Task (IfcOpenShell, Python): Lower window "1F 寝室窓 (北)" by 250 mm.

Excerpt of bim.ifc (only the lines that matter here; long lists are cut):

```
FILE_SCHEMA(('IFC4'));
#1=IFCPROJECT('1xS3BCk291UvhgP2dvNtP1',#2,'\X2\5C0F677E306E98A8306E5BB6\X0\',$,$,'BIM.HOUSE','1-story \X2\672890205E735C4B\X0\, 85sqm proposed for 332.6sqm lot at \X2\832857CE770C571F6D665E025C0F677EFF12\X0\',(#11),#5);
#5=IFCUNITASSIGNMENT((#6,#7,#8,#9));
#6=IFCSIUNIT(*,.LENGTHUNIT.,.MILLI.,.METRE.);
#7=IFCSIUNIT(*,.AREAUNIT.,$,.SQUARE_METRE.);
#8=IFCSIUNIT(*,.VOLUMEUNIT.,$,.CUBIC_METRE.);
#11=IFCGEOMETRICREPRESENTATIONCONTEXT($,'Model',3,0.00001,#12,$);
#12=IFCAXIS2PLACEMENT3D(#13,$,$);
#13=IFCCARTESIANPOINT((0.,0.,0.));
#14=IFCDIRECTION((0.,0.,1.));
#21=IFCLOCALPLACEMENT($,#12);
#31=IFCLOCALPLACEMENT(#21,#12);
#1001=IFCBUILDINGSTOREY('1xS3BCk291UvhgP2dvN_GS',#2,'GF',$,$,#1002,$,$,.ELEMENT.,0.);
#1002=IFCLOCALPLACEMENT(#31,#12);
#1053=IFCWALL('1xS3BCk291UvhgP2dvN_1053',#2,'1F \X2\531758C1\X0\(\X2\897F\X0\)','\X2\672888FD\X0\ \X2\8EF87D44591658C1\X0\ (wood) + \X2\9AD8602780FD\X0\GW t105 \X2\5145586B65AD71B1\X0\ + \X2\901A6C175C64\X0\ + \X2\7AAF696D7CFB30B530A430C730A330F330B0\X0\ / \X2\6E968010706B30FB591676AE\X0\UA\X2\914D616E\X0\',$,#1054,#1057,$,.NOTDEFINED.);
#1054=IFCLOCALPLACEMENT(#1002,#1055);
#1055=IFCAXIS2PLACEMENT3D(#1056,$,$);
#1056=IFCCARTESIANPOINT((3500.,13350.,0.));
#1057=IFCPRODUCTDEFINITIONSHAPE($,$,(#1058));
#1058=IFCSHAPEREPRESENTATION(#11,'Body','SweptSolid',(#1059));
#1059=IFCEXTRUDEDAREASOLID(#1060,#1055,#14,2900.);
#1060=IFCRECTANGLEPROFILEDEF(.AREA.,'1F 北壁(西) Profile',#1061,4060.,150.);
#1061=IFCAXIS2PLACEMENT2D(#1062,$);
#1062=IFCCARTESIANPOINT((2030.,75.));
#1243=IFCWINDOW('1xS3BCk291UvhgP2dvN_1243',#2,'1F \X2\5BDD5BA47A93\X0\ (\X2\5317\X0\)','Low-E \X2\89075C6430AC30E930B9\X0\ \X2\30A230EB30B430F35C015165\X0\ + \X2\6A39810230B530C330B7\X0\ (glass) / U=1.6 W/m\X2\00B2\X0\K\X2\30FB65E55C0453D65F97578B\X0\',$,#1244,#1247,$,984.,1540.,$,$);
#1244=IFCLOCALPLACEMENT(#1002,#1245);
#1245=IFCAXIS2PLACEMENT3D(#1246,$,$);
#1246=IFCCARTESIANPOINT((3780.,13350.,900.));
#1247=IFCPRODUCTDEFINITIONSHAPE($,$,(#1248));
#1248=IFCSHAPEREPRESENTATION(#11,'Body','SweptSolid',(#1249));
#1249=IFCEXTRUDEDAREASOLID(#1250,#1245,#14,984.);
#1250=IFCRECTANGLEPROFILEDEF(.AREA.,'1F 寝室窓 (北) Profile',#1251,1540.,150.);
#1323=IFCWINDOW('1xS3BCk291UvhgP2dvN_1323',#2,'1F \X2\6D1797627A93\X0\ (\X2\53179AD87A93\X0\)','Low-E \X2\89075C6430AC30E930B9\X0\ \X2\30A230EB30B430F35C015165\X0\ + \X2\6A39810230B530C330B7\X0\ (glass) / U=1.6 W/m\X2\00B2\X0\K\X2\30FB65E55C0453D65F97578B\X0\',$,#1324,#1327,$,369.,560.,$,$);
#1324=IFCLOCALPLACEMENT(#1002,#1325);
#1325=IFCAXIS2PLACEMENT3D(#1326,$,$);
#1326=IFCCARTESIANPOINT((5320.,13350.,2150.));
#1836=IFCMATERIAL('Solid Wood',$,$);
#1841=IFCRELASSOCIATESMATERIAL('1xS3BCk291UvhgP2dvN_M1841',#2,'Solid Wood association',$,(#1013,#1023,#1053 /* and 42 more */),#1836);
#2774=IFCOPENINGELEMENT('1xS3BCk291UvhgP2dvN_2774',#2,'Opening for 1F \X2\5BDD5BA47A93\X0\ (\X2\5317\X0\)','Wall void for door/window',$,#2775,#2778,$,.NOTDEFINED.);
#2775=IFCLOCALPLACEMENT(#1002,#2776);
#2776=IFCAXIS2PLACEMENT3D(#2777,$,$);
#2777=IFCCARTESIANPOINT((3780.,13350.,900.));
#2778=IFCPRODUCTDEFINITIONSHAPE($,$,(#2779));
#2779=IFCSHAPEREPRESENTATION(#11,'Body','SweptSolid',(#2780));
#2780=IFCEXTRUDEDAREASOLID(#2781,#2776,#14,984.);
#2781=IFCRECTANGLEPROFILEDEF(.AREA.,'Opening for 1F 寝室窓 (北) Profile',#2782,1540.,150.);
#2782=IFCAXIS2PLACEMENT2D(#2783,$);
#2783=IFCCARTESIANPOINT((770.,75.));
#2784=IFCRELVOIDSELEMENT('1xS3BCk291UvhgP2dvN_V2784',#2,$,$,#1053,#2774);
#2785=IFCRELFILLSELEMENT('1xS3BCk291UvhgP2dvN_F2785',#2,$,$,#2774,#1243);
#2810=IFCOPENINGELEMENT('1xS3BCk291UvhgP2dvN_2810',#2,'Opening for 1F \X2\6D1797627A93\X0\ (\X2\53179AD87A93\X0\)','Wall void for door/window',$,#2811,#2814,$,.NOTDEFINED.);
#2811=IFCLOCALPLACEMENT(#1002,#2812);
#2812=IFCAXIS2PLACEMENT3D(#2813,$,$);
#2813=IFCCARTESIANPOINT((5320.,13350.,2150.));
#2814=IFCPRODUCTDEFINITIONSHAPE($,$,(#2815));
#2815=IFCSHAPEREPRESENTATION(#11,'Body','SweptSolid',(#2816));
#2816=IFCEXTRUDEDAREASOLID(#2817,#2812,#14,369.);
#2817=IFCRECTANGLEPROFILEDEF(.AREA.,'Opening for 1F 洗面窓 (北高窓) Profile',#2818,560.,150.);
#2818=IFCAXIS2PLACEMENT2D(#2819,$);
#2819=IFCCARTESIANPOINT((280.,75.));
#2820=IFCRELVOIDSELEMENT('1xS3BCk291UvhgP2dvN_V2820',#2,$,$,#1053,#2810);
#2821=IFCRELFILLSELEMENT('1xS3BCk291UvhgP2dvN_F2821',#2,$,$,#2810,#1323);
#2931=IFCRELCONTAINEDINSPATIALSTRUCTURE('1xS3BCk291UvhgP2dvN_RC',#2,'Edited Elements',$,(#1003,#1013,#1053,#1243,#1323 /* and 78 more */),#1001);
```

```python
import numpy as np
import ifcopenshell
import ifcopenshell.api.geometry
import ifcopenshell.util.placement
import ifcopenshell.util.unit

model = ifcopenshell.open("bim.ifc")
unit_scale = ifcopenshell.util.unit.calculate_unit_scale(model)

window = model.by_guid("1xS3BCk291UvhgP2dvN_1243")
opening = window.FillsVoids[0].RelatingOpeningElement
dz = -0.25 / unit_scale

shift = np.array([0.0, 0.0, dz])
# The window is not placed relative to its opening, so move both.
for product in (opening, window):
    matrix = ifcopenshell.util.placement.get_local_placement(product.ObjectPlacement)
    matrix[:3, 3] += shift
    ifcopenshell.api.geometry.edit_object_placement(model, product=product, matrix=matrix, is_si=False)

print(f"moved by {dz * unit_scale:+.3f} m")

model.write("bim_v2.ifc")
```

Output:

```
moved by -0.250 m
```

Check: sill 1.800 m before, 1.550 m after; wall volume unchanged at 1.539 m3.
